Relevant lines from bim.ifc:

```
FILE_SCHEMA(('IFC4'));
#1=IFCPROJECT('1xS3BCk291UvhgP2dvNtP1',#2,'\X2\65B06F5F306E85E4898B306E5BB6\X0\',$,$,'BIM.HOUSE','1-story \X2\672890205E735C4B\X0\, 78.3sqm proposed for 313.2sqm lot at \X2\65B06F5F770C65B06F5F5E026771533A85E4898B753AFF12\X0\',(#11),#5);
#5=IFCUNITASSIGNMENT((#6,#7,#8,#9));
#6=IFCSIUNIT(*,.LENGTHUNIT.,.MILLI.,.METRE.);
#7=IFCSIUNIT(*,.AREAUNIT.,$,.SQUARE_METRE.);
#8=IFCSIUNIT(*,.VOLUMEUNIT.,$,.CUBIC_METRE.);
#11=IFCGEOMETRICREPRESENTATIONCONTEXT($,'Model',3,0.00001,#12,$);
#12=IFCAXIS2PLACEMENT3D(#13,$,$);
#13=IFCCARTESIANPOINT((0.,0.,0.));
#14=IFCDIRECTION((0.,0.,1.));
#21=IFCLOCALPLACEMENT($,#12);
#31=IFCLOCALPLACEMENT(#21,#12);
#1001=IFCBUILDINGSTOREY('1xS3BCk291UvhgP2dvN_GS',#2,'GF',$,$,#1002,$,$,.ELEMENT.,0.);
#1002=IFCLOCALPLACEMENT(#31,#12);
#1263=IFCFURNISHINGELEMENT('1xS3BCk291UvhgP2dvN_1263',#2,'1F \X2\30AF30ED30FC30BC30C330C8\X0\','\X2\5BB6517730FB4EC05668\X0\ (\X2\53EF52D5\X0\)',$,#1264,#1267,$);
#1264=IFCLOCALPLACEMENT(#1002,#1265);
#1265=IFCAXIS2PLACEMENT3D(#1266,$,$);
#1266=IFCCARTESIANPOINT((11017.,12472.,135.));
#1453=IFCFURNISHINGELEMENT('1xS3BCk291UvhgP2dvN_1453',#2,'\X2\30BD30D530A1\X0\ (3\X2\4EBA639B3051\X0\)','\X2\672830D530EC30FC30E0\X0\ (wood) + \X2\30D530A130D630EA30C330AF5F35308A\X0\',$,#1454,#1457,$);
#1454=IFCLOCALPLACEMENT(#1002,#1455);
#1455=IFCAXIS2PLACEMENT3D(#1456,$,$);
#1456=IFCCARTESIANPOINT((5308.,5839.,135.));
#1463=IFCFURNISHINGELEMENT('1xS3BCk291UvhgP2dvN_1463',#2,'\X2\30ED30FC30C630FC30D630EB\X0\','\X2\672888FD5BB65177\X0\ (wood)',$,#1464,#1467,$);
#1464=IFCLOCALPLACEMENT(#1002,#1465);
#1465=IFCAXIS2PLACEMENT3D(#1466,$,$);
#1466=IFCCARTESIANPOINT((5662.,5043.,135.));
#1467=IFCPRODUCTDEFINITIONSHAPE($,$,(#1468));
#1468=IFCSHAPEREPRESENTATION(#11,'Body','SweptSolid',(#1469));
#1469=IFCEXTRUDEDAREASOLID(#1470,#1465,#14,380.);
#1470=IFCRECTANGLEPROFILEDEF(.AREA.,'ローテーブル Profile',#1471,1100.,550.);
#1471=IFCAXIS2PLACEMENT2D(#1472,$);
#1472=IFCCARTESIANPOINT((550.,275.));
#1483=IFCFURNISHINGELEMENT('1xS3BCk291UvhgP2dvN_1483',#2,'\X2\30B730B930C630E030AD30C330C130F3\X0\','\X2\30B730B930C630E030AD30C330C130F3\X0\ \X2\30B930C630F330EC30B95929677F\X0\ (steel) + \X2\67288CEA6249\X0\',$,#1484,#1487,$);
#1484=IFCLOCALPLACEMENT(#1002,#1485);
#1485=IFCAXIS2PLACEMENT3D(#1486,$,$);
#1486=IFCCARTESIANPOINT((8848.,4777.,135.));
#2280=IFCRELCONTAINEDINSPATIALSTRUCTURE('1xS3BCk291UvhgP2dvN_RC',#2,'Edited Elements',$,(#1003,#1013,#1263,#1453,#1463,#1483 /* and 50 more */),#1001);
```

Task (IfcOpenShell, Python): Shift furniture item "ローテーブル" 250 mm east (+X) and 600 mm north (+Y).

```python
import ifcopenshell
import ifcopenshell.api.geometry
import ifcopenshell.util.placement
import ifcopenshell.util.unit

model = ifcopenshell.open("bim.ifc")
unit_scale = ifcopenshell.util.unit.calculate_unit_scale(model)

item = model.by_id(1463)
matrix = ifcopenshell.util.placement.get_local_placement(item.ObjectPlacement)
matrix[0, 3] += 0.25 / unit_scale
matrix[1, 3] += 0.6 / unit_scale
ifcopenshell.api.geometry.edit_object_placement(model, product=item, matrix=matrix, is_si=False)

print(ifcopenshell.util.placement.get_local_placement(item.ObjectPlacement).round(3) + 0.0)

model.write("bim_updated.ifc")
```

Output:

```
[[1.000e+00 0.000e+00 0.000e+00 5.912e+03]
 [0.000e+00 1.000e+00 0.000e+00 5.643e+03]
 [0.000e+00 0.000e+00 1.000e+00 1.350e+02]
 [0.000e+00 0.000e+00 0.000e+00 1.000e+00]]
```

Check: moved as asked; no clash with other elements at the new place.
